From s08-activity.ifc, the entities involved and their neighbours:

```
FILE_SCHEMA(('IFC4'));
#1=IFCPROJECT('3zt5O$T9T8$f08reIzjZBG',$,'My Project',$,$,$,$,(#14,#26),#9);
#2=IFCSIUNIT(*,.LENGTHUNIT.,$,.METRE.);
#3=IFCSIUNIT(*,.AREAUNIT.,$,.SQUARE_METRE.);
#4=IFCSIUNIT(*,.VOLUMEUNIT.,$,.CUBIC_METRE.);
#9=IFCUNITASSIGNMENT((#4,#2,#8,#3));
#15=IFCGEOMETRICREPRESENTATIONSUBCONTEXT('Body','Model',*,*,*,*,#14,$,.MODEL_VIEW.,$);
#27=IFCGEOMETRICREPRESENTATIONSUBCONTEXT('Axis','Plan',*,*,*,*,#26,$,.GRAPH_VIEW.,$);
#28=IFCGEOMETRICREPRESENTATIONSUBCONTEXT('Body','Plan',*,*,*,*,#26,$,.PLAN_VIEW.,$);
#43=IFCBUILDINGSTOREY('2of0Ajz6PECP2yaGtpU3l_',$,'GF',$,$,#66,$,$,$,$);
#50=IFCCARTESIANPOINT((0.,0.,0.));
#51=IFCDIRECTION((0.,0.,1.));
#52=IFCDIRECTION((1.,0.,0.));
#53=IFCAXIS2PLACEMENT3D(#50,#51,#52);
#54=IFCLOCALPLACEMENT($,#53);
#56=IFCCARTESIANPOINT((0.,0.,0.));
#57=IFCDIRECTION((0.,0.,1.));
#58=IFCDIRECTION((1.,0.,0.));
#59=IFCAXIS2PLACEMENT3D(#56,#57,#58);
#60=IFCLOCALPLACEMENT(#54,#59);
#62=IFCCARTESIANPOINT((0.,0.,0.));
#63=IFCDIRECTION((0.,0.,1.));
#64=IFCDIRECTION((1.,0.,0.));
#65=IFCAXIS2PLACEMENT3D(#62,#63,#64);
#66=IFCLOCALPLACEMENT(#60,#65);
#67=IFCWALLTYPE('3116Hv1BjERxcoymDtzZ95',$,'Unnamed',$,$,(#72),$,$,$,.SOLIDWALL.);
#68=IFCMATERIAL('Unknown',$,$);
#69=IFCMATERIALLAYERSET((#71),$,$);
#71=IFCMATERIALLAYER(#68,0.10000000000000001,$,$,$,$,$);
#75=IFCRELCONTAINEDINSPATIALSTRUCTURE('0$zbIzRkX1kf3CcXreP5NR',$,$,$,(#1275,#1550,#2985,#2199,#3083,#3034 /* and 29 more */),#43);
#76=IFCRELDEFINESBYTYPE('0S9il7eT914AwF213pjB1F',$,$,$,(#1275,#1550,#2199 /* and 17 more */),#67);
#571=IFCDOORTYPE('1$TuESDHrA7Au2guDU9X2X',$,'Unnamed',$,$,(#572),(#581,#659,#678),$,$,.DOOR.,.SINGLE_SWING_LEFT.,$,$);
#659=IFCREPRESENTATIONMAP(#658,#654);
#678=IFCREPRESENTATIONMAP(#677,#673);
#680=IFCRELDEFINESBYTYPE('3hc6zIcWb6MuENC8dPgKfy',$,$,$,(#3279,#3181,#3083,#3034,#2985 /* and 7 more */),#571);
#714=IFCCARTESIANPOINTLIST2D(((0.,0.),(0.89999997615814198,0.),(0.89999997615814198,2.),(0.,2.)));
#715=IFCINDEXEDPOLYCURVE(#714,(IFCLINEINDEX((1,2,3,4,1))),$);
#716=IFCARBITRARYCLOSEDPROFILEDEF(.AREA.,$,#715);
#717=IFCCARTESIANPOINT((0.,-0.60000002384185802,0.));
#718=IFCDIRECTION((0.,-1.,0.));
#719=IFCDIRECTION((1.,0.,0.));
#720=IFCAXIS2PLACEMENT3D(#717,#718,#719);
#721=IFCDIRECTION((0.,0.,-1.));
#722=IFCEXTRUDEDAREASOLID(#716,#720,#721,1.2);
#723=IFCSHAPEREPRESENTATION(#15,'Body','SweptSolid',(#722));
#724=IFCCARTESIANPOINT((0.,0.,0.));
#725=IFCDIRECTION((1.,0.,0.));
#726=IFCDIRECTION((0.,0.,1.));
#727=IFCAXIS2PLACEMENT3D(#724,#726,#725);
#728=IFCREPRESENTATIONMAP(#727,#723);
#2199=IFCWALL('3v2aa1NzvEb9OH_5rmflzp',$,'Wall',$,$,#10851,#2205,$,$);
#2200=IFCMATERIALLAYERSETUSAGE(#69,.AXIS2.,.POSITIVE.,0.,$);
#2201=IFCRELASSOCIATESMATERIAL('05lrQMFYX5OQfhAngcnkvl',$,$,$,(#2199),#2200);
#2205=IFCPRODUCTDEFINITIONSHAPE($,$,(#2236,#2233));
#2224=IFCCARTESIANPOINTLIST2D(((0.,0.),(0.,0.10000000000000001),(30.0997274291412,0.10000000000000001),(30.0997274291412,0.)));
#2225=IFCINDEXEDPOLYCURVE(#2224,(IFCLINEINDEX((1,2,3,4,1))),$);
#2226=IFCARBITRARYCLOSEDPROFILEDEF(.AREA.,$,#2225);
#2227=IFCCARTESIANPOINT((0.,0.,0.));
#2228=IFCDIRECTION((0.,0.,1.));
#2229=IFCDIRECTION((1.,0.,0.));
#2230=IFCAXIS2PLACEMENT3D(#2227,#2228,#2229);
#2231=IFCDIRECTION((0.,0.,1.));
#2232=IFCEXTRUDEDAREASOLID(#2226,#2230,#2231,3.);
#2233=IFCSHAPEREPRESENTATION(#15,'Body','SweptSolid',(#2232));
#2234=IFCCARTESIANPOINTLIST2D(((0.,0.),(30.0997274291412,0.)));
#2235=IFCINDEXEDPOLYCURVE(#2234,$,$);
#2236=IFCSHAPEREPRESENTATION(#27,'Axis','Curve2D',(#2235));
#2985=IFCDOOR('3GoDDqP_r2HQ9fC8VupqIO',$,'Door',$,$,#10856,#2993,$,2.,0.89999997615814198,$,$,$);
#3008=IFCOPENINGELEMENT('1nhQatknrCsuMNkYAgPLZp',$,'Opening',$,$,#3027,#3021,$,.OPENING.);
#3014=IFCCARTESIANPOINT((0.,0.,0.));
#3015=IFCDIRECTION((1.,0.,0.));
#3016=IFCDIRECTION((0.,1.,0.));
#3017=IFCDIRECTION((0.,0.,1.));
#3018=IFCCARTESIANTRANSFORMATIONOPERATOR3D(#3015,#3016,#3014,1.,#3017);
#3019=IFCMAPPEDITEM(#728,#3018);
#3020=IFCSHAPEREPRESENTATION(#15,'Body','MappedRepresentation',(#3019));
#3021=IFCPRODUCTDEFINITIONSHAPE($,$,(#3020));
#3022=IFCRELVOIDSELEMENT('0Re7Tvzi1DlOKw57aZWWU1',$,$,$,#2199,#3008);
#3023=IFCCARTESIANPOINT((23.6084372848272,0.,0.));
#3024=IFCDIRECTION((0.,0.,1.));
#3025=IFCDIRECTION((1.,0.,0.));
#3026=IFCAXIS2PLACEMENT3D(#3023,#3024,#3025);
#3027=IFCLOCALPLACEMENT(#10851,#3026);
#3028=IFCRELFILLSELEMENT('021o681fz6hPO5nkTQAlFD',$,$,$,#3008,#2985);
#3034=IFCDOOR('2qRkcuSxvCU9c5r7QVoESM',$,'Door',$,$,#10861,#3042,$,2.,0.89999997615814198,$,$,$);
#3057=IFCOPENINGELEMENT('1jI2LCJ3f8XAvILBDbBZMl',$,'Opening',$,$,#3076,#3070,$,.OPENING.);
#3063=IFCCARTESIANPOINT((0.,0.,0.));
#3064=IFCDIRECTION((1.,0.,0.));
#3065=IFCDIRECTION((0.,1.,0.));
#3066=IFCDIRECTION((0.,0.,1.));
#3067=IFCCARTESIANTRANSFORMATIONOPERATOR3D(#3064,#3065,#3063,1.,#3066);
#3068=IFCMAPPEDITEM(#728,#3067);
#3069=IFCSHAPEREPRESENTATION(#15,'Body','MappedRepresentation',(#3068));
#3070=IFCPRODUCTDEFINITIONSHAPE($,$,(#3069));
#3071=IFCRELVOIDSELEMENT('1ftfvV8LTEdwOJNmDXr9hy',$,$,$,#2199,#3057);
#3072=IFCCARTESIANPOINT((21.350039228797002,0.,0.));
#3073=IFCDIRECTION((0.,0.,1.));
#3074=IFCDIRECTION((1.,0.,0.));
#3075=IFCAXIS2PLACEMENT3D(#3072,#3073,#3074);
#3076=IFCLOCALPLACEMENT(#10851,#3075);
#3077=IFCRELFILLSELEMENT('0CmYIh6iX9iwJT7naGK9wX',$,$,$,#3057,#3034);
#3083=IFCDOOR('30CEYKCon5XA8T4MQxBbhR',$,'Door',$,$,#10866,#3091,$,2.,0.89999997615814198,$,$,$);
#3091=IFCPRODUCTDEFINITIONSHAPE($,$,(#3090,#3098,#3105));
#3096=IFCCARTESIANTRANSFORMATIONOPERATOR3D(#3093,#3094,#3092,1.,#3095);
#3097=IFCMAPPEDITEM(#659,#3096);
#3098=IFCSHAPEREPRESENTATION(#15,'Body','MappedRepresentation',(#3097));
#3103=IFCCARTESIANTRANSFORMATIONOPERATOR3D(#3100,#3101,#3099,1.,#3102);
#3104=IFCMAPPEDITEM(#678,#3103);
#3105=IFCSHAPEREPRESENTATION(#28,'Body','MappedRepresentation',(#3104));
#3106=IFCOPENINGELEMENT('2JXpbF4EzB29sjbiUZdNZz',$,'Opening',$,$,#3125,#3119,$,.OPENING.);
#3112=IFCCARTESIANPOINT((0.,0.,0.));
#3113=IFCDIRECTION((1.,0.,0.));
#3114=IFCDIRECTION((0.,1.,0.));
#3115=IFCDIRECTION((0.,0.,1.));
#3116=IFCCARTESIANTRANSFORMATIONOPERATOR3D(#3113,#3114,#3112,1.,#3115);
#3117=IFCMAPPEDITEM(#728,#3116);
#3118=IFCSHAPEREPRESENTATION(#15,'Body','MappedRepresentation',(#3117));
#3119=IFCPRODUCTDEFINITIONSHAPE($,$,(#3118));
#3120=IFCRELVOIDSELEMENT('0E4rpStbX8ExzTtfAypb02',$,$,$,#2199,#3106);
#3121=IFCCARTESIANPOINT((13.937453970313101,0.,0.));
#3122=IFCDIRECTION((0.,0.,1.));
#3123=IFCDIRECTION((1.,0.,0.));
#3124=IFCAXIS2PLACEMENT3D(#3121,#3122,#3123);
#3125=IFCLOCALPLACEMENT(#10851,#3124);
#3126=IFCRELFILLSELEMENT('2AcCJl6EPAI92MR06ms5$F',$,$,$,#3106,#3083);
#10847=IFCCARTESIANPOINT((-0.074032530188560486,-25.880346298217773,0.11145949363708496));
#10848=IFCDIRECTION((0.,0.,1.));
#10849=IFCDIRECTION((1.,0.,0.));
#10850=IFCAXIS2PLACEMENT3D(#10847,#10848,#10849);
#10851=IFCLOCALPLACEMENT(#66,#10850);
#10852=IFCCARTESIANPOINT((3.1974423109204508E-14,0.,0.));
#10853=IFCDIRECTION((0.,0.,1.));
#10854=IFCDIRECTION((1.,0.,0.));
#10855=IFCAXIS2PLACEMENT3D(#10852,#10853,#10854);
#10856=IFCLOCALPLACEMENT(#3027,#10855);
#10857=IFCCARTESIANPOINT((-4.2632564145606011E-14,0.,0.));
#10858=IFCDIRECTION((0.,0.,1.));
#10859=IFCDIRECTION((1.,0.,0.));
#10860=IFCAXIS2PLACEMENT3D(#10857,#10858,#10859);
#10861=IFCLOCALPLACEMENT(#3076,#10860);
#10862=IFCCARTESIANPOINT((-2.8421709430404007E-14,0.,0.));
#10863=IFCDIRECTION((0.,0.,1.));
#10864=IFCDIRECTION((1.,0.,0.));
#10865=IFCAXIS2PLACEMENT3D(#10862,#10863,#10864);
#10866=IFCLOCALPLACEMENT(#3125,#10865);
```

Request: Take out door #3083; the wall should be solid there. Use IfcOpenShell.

```python
import ifcopenshell
import ifcopenshell.api.feature
import ifcopenshell.api.root
import ifcopenshell.geom
import ifcopenshell.util.shape

model = ifcopenshell.open("s08-activity.ifc")
settings = ifcopenshell.geom.settings()


def volume(element):
    """Net volume in cubic metres, openings subtracted."""
    shape = ifcopenshell.geom.create_shape(settings, element)
    return ifcopenshell.util.shape.get_volume(shape.geometry)


door = model.by_guid("30CEYKCon5XA8T4MQxBbhR")
opening = door.FillsVoids[0].RelatingOpeningElement
wall = opening.VoidsElements[0].RelatingBuildingElement
before = volume(wall)

ifcopenshell.api.root.remove_product(model, product=door)
ifcopenshell.api.feature.remove_feature(model, feature=opening)

after = volume(wall)

print(f"wall volume {before:.3f} -> {after:.3f} m3")

model.write("s08-activity_rev.ifc")
```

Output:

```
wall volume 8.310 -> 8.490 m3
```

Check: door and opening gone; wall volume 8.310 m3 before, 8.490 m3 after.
